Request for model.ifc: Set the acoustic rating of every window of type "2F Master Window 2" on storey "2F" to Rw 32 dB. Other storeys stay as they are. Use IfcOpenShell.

First a look at what the model holds.

```python
import ifcopenshell
import ifcopenshell.util.element

model = ifcopenshell.open("model.ifc")
print(model.schema)
storey = next(s for s in model.by_type("IfcBuildingStorey") if s.Name == "2F")
windows = [e for e in ifcopenshell.util.element.get_decomposition(storey) if e.is_a("IfcWindow")]
seen = {}
for e in windows:
    element_type = ifcopenshell.util.element.get_type(e)
    key = (element_type.Name if element_type != e and element_type else None, ifcopenshell.util.element.get_pset(e, "Pset_WindowCommon", "AcousticRating"))
    seen[key] = seen.get(key, 0) + 1
for (name, value), count in sorted(seen.items(), key=str):
    print(count, "x", name, "|", value)
```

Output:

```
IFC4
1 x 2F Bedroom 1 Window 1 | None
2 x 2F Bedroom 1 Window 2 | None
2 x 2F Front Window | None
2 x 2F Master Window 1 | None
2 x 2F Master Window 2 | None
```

```python
import ifcopenshell
import ifcopenshell.api.pset
import ifcopenshell.util.element

model = ifcopenshell.open("model.ifc")

storey = next(s for s in model.by_type("IfcBuildingStorey") if s.Name == "2F")
windows = [e for e in ifcopenshell.util.element.get_decomposition(storey) if e.is_a("IfcWindow")]

count = 0
for e in windows:
    element_type = ifcopenshell.util.element.get_type(e)
    if element_type in (None, e) or element_type.Name != "2F Master Window 2":
        continue
    # add_pset returns the element's existing set when there is one.
    pset = ifcopenshell.api.pset.add_pset(model, product=e, name="Pset_WindowCommon")
    ifcopenshell.api.pset.edit_pset(model, pset=pset, properties={"AcousticRating": "Rw 32 dB"})
    count += 1

print(count, "windows updated")

model.write("model_updated.ifc")
```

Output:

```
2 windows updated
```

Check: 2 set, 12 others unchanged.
